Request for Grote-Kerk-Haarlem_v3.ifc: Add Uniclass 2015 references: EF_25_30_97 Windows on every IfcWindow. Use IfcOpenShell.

First a look at what the model holds.

```python
import ifcopenshell

model = ifcopenshell.open("Grote-Kerk-Haarlem_v3.ifc")
print(model.schema)
print("classifications:", [c.Name for c in model.by_type("IfcClassification")])
for ifc_class in ("IfcDoor", "IfcRoof", "IfcStair", "IfcWall", "IfcWindow"):
    print(ifc_class, len(model.by_type(ifc_class)))
```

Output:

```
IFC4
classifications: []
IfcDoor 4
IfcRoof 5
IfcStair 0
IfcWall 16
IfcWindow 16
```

```python
import ifcopenshell
import ifcopenshell.api.classification

model = ifcopenshell.open("Grote-Kerk-Haarlem_v3.ifc")

system = ifcopenshell.api.classification.add_classification(model, classification="Uniclass 2015")

codes = {
    "IfcWindow": ("EF_25_30_97", "Windows"),
}
for ifc_class, (code, name) in codes.items():
    products = model.by_type(ifc_class)
    ifcopenshell.api.classification.add_reference(
        model, products=products, classification=system, identification=code, name=name
    )
    print(code, len(products))

model.write("Grote-Kerk-Haarlem_v3_updated.ifc")
```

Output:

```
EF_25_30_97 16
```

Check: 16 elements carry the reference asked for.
